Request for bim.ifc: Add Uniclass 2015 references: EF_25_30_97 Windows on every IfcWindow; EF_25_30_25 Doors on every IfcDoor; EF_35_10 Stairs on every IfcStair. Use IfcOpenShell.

First a look at what the model holds.

```python
import ifcopenshell

model = ifcopenshell.open("bim.ifc")
print(model.schema)
print("classifications:", [c.Name for c in model.by_type("IfcClassification")])
for ifc_class in ("IfcDoor", "IfcRoof", "IfcStair", "IfcWall", "IfcWindow"):
    print(ifc_class, len(model.by_type(ifc_class)))
```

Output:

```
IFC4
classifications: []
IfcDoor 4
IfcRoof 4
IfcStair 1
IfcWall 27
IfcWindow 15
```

```python
import ifcopenshell
import ifcopenshell.api.classification

model = ifcopenshell.open("bim.ifc")

system = ifcopenshell.api.classification.add_classification(model, classification="Uniclass 2015")

codes = {
    "IfcWindow": ("EF_25_30_97", "Windows"),
    "IfcDoor": ("EF_25_30_25", "Doors"),
    "IfcStair": ("EF_35_10", "Stairs"),
}
for ifc_class, (code, name) in codes.items():
    products = model.by_type(ifc_class)
    ifcopenshell.api.classification.add_reference(
        model, products=products, classification=system, identification=code, name=name
    )
    print(code, len(products))

model.write("bim_updated.ifc")
```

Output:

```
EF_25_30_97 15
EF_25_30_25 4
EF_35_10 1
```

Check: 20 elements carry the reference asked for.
